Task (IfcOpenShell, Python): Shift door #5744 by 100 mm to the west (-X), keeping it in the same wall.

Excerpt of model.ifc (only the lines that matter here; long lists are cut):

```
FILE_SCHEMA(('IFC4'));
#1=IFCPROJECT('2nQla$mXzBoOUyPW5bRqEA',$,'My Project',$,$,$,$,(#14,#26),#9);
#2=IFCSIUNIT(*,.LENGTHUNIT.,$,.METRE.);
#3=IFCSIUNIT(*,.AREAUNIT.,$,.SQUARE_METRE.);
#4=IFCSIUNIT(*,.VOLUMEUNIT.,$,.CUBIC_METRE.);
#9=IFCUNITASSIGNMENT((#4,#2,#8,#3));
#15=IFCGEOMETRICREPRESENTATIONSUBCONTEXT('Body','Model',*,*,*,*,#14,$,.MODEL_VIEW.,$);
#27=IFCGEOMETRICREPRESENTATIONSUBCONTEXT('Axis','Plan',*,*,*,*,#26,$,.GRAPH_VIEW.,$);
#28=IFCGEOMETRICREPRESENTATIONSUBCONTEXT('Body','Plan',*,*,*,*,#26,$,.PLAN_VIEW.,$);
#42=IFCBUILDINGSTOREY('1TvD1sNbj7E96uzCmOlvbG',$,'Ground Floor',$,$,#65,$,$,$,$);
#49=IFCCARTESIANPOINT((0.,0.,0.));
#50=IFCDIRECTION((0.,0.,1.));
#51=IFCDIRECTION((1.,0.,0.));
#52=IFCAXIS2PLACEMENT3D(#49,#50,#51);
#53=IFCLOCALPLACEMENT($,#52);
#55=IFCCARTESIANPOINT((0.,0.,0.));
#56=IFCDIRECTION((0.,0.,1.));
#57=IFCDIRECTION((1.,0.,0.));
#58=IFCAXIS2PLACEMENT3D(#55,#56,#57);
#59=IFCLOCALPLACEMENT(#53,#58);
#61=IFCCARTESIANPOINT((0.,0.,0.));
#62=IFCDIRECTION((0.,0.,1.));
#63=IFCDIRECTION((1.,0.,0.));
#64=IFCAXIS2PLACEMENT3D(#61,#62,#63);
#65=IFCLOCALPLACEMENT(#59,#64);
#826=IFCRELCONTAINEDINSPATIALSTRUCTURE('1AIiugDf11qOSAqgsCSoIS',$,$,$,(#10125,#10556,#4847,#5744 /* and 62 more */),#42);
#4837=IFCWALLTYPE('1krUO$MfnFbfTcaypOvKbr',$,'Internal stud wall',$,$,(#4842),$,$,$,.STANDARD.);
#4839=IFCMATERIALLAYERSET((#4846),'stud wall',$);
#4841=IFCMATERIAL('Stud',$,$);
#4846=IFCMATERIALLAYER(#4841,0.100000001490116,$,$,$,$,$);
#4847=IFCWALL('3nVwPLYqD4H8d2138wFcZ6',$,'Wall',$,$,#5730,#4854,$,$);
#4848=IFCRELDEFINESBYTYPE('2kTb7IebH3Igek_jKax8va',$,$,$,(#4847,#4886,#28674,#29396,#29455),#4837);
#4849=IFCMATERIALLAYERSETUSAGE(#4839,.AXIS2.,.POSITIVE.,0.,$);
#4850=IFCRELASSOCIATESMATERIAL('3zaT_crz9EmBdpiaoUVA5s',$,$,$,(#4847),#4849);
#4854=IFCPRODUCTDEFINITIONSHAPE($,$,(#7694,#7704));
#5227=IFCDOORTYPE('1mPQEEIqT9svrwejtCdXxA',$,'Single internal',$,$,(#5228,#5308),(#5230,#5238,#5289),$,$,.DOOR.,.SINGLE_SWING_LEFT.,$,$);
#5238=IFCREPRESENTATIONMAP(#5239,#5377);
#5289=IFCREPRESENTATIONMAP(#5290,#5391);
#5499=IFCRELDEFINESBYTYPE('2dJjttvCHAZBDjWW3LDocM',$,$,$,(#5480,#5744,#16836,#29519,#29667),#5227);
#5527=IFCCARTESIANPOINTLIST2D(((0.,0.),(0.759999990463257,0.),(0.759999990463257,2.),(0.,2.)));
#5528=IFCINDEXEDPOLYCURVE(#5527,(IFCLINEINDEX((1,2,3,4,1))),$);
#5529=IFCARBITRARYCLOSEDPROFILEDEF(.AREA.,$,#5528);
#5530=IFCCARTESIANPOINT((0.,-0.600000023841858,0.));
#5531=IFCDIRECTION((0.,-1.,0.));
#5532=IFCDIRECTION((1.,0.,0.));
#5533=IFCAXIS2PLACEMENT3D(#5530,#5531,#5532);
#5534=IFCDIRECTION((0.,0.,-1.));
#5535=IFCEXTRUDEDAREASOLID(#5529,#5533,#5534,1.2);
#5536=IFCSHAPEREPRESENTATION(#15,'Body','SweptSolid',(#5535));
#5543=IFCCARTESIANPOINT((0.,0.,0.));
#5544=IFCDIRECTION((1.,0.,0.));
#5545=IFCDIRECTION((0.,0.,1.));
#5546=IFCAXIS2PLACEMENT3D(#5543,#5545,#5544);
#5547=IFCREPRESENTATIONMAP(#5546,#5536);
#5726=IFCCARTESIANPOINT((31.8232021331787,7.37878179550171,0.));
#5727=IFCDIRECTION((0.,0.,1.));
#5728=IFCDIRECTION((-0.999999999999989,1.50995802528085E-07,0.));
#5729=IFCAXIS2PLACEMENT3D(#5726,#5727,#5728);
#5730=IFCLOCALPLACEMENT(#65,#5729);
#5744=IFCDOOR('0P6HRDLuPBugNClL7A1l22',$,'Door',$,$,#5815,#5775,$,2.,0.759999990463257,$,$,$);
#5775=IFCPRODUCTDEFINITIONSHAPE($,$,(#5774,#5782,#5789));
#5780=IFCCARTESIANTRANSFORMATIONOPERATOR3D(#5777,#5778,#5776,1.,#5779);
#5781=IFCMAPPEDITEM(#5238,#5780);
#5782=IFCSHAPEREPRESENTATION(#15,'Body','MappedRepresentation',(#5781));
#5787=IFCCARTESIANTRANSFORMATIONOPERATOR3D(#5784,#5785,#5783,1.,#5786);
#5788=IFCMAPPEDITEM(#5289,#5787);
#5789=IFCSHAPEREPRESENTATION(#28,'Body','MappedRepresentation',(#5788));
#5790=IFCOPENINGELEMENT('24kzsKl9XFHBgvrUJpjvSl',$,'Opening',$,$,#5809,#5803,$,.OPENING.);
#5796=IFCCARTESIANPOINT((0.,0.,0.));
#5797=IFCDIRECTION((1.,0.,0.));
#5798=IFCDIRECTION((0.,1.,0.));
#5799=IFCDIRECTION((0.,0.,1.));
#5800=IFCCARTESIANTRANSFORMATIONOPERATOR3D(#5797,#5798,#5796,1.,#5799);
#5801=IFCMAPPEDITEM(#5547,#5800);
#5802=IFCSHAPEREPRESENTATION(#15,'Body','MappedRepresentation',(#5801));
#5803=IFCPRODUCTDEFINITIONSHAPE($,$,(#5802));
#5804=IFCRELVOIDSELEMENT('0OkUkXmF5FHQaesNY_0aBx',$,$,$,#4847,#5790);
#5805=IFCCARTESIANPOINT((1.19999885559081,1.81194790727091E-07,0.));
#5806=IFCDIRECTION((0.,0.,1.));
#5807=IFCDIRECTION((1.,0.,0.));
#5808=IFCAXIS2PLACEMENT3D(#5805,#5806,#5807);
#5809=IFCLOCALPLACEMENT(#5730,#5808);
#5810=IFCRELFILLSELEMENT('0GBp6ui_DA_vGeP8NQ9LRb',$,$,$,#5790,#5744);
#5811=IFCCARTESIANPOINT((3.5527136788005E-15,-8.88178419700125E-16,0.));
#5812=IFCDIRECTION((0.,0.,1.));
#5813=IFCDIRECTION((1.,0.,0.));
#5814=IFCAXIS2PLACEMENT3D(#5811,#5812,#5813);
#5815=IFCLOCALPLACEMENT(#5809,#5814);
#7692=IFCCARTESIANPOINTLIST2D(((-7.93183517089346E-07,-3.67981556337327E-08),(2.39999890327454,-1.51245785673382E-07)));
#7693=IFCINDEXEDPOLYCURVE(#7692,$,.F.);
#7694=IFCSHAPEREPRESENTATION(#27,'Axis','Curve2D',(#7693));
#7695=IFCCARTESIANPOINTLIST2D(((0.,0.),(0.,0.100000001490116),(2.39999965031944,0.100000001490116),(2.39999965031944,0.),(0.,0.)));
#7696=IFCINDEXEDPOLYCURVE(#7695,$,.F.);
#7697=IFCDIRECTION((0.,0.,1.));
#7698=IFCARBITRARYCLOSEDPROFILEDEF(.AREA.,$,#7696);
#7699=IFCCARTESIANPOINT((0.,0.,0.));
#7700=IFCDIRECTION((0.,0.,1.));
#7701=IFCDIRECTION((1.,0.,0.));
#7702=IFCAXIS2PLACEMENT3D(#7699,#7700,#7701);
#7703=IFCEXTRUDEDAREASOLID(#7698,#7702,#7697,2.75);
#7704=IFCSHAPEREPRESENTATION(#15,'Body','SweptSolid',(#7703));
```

```python
import ifcopenshell
import ifcopenshell.api.geometry
import ifcopenshell.util.placement

model = ifcopenshell.open("model.ifc")

door = model.by_guid("0P6HRDLuPBugNClL7A1l22")
opening = door.FillsVoids[0].RelatingOpeningElement
wall = opening.VoidsElements[0].RelatingBuildingElement

wall_matrix = ifcopenshell.util.placement.get_local_placement(wall.ObjectPlacement)
shift = wall_matrix[:3, 0] * 0.1
before = ifcopenshell.util.placement.get_local_placement(door.ObjectPlacement)[:3, 3].copy()

# The door is placed relative to its opening, so it follows when the opening moves.
matrix = ifcopenshell.util.placement.get_local_placement(opening.ObjectPlacement)
matrix[:3, 3] += shift
ifcopenshell.api.geometry.edit_object_placement(
    model, product=opening, matrix=matrix, is_si=False, should_transform_children=True
)

after = ifcopenshell.util.placement.get_local_placement(door.ObjectPlacement)[:3, 3]
print("door moved by", (after - before).round(3) + 0.0)

model.write("model-out.ifc")
```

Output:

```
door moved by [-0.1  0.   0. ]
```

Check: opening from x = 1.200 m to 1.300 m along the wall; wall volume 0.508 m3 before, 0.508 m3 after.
